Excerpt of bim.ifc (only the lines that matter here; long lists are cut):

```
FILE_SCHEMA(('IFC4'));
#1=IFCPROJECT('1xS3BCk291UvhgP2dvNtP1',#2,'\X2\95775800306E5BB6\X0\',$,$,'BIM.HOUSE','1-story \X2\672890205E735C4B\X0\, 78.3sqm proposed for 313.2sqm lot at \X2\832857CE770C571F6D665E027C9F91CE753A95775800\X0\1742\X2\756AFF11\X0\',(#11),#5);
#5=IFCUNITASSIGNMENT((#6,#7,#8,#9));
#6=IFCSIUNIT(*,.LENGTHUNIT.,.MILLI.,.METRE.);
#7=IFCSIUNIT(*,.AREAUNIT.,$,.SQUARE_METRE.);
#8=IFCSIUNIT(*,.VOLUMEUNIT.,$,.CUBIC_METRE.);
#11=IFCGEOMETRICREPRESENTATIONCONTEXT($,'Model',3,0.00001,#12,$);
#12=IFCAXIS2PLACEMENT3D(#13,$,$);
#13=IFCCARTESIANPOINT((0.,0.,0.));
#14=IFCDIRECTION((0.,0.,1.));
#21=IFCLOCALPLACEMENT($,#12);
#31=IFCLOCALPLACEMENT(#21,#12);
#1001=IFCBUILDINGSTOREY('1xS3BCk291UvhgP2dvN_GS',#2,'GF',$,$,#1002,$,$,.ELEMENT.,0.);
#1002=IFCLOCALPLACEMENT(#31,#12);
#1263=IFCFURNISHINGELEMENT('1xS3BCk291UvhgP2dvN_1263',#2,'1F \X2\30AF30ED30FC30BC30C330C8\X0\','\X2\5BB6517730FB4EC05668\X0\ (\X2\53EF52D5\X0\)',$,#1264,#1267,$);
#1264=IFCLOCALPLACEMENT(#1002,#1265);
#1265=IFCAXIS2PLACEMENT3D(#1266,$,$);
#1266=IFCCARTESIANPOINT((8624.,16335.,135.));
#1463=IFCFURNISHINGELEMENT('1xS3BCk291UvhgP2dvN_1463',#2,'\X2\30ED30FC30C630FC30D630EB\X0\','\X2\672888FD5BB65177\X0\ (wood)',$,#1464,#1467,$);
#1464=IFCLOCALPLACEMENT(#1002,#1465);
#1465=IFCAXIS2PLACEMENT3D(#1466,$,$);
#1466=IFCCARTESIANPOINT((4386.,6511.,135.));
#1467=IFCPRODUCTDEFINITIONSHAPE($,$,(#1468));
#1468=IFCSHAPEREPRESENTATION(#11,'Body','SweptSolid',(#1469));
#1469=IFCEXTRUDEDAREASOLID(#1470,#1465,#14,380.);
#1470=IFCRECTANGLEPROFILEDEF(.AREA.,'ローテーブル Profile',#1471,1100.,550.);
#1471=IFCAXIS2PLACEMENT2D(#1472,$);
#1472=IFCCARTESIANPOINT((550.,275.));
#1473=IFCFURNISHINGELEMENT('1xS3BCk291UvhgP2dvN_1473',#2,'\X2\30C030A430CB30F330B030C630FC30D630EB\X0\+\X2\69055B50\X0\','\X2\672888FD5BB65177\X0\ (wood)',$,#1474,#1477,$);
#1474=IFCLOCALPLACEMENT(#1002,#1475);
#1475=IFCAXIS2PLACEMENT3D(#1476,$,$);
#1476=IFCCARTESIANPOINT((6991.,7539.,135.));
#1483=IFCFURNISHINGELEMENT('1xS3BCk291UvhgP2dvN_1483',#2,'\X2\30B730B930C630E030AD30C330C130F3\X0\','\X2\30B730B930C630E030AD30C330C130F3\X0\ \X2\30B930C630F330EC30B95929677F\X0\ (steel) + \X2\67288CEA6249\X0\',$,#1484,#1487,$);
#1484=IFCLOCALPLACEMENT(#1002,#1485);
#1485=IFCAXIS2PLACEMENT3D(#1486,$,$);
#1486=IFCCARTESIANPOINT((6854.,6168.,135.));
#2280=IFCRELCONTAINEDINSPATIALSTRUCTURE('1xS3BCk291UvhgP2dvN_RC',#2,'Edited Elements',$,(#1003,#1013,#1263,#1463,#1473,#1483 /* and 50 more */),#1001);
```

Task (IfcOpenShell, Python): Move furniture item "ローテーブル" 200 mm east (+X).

```python
import ifcopenshell
import ifcopenshell.api.geometry
import ifcopenshell.util.placement

model = ifcopenshell.open("bim.ifc")

item = model.by_id(1463)
matrix = ifcopenshell.util.placement.get_local_placement(item.ObjectPlacement)
matrix[0, 3] += 200.0
ifcopenshell.api.geometry.edit_object_placement(model, product=item, matrix=matrix, is_si=False)

print(ifcopenshell.util.placement.get_local_placement(item.ObjectPlacement).round(3) + 0.0)

model.write("bim_updated.ifc")
```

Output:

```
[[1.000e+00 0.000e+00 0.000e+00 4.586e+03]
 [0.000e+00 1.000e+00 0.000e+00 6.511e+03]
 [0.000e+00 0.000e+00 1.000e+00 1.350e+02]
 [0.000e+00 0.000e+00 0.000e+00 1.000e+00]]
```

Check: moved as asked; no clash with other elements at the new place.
